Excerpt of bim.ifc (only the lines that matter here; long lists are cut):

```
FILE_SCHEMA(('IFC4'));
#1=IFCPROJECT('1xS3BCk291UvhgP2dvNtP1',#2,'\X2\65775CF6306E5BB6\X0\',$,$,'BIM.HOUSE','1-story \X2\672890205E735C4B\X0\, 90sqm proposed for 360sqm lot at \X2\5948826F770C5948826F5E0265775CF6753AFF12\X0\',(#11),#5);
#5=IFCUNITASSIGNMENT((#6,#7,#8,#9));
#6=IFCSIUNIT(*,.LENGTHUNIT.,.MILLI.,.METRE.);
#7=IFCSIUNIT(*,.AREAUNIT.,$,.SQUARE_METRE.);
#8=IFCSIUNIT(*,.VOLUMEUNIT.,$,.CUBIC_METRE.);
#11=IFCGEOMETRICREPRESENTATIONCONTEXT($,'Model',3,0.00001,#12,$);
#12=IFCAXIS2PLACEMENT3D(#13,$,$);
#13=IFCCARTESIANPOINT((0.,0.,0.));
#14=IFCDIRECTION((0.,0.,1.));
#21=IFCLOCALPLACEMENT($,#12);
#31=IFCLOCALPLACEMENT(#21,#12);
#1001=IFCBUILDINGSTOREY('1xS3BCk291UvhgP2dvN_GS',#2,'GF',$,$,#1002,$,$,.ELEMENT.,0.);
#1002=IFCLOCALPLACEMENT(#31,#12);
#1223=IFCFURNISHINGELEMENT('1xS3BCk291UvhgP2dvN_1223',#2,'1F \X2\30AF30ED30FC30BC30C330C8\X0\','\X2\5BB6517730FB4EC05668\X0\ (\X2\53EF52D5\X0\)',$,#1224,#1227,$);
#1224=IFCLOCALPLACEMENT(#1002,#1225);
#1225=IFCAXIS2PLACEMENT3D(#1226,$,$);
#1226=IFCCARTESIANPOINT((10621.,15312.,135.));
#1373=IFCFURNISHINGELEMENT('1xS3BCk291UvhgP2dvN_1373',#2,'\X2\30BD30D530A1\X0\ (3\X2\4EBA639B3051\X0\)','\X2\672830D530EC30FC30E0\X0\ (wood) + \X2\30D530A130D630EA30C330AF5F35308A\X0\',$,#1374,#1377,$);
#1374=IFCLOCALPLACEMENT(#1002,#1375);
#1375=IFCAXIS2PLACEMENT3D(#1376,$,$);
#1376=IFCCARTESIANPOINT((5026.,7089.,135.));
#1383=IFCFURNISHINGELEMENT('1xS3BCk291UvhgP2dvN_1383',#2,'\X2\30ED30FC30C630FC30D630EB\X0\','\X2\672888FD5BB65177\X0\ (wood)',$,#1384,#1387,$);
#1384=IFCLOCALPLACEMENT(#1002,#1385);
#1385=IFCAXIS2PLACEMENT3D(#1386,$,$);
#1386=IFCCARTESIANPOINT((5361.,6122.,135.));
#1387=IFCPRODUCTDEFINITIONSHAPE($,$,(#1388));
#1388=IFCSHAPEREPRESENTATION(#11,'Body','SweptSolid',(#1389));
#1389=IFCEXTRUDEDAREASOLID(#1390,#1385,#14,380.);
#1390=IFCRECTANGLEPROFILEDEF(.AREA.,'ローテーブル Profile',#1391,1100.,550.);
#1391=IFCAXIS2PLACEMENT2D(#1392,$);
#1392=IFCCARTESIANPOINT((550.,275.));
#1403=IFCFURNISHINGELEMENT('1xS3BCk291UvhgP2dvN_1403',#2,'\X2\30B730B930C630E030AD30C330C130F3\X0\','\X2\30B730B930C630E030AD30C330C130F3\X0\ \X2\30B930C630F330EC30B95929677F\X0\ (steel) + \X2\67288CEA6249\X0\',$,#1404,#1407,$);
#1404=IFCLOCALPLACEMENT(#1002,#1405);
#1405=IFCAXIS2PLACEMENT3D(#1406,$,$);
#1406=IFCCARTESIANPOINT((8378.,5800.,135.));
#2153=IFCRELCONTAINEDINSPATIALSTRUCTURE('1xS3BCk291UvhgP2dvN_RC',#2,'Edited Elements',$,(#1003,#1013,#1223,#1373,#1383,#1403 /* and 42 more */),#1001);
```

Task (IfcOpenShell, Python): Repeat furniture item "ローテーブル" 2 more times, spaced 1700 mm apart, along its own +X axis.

```python
import ifcopenshell
import ifcopenshell.api.geometry
import ifcopenshell.api.root
import ifcopenshell.util.element
import ifcopenshell.util.placement

model = ifcopenshell.open("bim.ifc")


def reuse_history(source, copy):
    """copy_class also copies each property set's owner history, people and application; keep the originals."""
    for rel in copy.IsDefinedBy:
        if rel.is_a("IfcRelDefinesByProperties") and (history := rel.RelatingPropertyDefinition.OwnerHistory):
            rel.RelatingPropertyDefinition.OwnerHistory = source.OwnerHistory
            ifcopenshell.util.element.remove_deep2(model, history)


source = model.by_id(1383)
base = ifcopenshell.util.placement.get_local_placement(source.ObjectPlacement)
step = base[:3, 0] * 1700.0

for i in range(1, 3):
    copy = ifcopenshell.api.root.copy_class(model, product=source)
    copy.Representation = ifcopenshell.util.element.copy_deep(
        model, source.Representation, exclude=["IfcGeometricRepresentationContext", "IfcRepresentationMap"]
    )
    reuse_history(source, copy)
    matrix = base.copy()
    matrix[:3, 3] += i * step
    print("added at", matrix[:3, 3].round(3) + 0.0)
    ifcopenshell.api.geometry.edit_object_placement(model, product=copy, matrix=matrix, is_si=False)

model.write("bim-out.ifc")
```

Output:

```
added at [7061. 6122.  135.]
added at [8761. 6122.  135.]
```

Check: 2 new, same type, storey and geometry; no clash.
